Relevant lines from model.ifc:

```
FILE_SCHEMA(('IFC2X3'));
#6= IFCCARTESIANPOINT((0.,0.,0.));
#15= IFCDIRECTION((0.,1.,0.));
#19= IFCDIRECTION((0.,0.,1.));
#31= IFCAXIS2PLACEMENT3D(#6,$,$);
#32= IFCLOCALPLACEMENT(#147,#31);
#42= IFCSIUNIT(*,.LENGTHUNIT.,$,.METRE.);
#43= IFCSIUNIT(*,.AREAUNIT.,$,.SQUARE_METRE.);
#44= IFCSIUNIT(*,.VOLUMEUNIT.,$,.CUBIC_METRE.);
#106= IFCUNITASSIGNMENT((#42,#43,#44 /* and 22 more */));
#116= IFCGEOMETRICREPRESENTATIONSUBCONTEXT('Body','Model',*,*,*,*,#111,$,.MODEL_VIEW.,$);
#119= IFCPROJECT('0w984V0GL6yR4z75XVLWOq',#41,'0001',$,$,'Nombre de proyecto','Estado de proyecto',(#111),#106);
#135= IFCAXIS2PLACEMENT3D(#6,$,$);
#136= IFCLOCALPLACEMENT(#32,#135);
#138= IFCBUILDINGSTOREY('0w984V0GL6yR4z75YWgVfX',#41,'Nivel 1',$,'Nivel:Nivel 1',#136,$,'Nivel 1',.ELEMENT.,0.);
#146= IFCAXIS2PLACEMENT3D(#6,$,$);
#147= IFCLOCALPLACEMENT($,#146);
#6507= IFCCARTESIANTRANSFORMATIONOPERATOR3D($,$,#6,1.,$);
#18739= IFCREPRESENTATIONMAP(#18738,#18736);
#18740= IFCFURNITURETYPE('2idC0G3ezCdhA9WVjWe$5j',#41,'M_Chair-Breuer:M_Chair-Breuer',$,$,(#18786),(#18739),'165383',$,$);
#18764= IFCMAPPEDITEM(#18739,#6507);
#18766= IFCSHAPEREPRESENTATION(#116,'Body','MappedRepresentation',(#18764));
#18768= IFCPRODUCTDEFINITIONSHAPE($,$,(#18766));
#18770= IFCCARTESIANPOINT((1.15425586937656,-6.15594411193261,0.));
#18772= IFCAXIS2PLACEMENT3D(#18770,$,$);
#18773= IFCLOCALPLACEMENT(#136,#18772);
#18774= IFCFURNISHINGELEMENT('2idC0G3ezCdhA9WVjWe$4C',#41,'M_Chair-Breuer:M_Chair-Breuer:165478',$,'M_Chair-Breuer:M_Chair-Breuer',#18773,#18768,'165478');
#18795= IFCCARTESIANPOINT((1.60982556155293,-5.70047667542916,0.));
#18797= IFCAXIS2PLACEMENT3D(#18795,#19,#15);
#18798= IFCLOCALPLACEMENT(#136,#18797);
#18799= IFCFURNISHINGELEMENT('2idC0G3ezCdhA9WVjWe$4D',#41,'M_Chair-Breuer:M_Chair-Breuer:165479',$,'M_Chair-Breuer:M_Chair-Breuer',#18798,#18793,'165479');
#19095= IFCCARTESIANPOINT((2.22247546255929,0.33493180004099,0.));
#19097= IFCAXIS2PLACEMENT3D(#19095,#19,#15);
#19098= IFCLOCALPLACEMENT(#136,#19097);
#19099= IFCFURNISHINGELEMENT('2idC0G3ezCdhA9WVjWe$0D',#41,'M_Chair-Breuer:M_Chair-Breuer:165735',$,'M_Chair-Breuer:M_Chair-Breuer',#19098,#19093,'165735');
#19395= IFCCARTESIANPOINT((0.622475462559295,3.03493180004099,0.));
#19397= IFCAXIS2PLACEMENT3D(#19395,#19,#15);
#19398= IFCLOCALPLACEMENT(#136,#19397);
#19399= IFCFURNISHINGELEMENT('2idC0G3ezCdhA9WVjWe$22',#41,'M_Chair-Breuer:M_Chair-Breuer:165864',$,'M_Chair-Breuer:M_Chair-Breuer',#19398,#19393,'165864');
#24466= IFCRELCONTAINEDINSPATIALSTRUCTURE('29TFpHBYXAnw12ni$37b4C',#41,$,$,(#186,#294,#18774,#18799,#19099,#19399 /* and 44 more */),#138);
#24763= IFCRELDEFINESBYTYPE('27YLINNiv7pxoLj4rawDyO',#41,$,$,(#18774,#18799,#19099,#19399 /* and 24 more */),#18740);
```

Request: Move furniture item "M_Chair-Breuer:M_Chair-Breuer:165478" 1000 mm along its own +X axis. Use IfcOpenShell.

```python
import ifcopenshell
import ifcopenshell.api.geometry
import ifcopenshell.util.placement
import ifcopenshell.util.unit

model = ifcopenshell.open("model.ifc")
unit_scale = ifcopenshell.util.unit.calculate_unit_scale(model)

item = model.by_guid("2idC0G3ezCdhA9WVjWe$4C")
matrix = ifcopenshell.util.placement.get_local_placement(item.ObjectPlacement)
matrix[:3, 3] += matrix[:3, 0] * 1 / unit_scale
ifcopenshell.api.geometry.edit_object_placement(model, product=item, matrix=matrix, is_si=False)

print(ifcopenshell.util.placement.get_local_placement(item.ObjectPlacement).round(3) + 0.0)

model.write("model_v2.ifc")
```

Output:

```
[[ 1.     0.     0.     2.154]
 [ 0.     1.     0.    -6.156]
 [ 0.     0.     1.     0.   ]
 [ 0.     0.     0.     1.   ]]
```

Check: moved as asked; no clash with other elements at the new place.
